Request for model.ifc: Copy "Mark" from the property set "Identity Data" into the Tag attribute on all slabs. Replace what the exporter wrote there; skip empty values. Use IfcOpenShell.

First a look at what the model holds.

```python
import ifcopenshell
import ifcopenshell.util.element

model = ifcopenshell.open("model.ifc")
print(model.schema)
slabs = model.by_type("IfcSlab")
print(len(slabs), "slabs")
for e in slabs[:8]:
    source = ifcopenshell.util.element.get_pset(e, "Identity Data", "Mark")
    target = e.Tag
    print(e.id(), repr(source), repr(target), sep=" | ")
```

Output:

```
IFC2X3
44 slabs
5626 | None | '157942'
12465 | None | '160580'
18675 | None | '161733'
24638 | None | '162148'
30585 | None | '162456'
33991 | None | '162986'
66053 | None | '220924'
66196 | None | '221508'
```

```python
import ifcopenshell
import ifcopenshell.util.element

model = ifcopenshell.open("model.ifc")

count = 0
for e in model.by_type("IfcSlab"):
    value = ifcopenshell.util.element.get_pset(e, "Identity Data", "Mark")
    current = e.Tag
    if not value or not value.strip() or current == value:
        continue
    e.Tag = value
    count += 1

print(count, "slabs updated")

model.write("model_rev.ifc")
```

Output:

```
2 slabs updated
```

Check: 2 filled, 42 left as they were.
